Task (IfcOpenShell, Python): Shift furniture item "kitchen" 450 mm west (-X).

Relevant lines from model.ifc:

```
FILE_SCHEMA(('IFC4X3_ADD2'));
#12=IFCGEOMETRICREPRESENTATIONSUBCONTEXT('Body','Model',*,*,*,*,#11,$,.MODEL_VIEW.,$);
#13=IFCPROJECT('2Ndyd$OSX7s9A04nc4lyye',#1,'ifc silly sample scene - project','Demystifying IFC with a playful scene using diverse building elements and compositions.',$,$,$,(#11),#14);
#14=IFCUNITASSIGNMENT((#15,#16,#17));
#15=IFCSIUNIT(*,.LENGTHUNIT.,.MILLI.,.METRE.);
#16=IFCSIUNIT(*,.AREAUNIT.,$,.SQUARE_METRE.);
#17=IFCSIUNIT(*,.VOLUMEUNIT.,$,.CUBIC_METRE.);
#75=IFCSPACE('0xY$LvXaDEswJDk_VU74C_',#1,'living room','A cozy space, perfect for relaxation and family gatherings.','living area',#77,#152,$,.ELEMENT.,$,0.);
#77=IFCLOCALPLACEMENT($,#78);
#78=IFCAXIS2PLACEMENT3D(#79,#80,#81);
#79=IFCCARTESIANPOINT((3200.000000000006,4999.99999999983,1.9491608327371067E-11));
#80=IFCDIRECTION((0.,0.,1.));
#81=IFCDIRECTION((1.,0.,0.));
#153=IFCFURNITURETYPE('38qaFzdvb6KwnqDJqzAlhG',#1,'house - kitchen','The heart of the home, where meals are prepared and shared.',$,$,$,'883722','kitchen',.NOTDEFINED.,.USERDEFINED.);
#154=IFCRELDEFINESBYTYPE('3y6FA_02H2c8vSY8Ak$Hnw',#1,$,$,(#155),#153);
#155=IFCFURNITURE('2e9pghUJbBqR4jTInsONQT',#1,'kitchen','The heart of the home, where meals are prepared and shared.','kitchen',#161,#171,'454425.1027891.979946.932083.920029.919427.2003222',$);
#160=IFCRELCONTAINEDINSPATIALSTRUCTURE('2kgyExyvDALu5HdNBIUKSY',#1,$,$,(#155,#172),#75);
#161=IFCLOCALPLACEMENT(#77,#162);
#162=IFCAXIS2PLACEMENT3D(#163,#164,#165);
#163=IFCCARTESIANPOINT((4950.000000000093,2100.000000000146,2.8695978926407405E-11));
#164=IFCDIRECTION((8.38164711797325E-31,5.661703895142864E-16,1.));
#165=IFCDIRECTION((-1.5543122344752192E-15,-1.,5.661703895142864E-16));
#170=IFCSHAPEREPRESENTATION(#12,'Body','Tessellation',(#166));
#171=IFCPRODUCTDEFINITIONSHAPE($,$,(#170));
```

```python
import ifcopenshell
import ifcopenshell.api.geometry
import ifcopenshell.util.placement

model = ifcopenshell.open("model.ifc")

item = model.by_id(155)
matrix = ifcopenshell.util.placement.get_local_placement(item.ObjectPlacement)
matrix[0, 3] -= 450.0
ifcopenshell.api.geometry.edit_object_placement(model, product=item, matrix=matrix, is_si=False)

print(ifcopenshell.util.placement.get_local_placement(item.ObjectPlacement).round(3) + 0.0)

model.write("model-out.ifc")
```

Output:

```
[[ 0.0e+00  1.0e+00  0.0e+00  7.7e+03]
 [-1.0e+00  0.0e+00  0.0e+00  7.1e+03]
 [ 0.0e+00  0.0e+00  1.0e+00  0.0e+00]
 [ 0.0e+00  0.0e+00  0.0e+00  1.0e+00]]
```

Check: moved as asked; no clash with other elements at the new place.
